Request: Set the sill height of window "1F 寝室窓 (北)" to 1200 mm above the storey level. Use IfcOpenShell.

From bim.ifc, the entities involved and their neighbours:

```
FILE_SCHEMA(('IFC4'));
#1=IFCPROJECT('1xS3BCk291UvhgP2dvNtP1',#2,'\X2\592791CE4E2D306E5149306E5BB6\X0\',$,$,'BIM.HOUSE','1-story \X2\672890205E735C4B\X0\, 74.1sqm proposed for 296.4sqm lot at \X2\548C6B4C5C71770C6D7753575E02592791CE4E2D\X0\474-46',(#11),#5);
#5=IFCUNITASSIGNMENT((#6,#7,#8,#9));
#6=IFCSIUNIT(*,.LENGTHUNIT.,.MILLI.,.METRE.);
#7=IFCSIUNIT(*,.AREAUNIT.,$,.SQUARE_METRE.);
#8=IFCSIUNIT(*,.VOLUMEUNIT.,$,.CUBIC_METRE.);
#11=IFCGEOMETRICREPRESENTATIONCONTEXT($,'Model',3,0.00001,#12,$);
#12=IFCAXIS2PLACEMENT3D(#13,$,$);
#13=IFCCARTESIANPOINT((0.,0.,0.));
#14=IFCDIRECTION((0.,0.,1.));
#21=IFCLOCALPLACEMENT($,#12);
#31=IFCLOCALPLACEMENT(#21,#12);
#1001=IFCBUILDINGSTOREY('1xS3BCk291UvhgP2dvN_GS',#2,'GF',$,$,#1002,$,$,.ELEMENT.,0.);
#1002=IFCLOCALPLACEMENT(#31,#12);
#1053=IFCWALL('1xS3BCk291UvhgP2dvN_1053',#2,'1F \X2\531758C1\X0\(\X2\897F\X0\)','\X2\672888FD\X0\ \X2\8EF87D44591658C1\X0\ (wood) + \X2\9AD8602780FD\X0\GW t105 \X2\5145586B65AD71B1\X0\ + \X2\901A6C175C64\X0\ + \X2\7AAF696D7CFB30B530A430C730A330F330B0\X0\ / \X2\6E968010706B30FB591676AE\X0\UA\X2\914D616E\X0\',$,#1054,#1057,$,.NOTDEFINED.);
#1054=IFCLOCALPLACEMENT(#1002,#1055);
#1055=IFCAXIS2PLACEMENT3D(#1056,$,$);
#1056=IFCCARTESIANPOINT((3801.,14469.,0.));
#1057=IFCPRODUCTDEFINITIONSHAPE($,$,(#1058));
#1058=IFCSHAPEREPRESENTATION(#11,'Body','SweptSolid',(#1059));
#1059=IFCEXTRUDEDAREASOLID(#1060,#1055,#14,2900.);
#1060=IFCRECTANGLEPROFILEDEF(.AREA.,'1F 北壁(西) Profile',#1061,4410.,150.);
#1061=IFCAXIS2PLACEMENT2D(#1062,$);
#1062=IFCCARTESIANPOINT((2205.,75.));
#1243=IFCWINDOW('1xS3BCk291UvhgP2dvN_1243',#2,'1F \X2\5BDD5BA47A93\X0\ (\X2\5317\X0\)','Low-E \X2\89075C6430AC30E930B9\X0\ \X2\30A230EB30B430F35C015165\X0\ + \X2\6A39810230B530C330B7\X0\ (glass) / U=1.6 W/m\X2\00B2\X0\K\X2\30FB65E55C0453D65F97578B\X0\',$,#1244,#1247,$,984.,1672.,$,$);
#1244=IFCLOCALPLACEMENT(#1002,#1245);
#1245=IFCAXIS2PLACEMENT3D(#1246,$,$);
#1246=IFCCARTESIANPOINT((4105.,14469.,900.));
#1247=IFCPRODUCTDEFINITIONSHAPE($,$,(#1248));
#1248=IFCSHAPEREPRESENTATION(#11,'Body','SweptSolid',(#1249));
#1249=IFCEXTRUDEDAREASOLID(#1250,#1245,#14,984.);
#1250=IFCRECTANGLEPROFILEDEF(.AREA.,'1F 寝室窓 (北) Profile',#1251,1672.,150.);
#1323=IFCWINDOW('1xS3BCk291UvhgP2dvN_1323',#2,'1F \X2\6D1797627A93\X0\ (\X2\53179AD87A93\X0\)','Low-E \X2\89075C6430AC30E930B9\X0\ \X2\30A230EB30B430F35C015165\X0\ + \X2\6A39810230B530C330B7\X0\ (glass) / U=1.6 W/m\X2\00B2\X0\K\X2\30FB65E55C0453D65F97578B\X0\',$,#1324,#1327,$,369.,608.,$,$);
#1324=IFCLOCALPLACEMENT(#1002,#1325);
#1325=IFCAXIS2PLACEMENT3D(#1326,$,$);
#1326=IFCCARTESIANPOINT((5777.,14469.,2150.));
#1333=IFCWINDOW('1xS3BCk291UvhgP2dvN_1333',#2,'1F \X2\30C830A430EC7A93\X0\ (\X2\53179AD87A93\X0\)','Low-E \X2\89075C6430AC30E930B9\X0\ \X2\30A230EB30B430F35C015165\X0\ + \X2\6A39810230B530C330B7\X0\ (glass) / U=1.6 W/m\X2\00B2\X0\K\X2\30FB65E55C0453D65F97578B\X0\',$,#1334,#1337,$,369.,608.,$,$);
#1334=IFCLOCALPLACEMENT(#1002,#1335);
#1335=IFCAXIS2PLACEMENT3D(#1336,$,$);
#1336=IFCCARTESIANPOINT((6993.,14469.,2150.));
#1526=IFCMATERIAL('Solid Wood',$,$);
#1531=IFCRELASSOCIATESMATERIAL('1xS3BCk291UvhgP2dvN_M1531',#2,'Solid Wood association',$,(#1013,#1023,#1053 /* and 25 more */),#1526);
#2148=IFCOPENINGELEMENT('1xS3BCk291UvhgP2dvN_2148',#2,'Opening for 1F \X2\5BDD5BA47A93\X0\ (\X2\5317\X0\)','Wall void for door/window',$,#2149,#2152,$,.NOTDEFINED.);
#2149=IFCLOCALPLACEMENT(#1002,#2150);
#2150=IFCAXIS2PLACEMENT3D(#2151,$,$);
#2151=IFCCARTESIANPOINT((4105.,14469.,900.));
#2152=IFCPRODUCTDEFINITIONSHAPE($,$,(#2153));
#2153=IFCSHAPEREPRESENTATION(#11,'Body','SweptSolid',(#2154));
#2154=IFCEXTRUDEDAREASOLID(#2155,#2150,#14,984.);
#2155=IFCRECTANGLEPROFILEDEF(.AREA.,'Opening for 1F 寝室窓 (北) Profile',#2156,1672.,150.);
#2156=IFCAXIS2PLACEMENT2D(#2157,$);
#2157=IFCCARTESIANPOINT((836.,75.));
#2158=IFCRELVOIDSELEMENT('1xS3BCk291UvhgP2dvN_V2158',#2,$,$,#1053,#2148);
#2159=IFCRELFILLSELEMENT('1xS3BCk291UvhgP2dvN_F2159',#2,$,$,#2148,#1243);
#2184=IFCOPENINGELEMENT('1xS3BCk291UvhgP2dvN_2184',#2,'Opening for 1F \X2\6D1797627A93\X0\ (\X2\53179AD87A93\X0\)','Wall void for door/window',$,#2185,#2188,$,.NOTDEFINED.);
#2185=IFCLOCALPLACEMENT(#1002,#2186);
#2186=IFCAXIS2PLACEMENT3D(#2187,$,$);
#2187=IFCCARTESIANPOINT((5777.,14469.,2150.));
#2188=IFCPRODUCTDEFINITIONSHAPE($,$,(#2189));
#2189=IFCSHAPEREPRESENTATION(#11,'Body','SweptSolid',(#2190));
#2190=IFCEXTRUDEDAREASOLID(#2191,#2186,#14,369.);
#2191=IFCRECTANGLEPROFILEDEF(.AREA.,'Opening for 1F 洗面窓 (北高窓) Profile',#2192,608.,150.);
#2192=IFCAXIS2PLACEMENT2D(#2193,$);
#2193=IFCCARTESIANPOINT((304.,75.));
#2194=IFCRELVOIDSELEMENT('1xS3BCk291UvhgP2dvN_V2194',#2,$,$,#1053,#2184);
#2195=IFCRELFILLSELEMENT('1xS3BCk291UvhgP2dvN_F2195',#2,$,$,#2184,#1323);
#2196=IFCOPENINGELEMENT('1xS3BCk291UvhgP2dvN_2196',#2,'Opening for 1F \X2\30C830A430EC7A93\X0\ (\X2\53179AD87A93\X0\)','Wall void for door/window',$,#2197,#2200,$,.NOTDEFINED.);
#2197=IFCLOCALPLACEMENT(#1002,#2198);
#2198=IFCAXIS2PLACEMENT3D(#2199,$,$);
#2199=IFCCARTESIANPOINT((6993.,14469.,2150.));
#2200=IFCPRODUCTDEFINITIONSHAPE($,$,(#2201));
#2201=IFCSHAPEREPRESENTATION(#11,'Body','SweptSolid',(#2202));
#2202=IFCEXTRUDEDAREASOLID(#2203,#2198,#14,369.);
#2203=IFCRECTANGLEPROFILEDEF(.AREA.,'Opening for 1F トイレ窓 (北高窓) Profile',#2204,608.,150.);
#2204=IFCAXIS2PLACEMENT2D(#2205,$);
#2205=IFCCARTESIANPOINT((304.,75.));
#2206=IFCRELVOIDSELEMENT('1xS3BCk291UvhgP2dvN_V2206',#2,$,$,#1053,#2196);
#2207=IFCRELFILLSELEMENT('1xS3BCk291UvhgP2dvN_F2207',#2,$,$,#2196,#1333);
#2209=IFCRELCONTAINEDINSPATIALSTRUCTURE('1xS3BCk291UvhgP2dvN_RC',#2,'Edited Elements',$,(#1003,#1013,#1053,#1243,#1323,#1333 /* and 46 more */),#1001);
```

```python
import numpy as np
import ifcopenshell
import ifcopenshell.api.geometry
import ifcopenshell.geom
import ifcopenshell.util.element
import ifcopenshell.util.placement
import ifcopenshell.util.shape
import ifcopenshell.util.unit

model = ifcopenshell.open("bim.ifc")
unit_scale = ifcopenshell.util.unit.calculate_unit_scale(model)

window = model.by_guid("1xS3BCk291UvhgP2dvN_1243")
opening = window.FillsVoids[0].RelatingOpeningElement
storey = ifcopenshell.util.element.get_container(window, ifc_class="IfcBuildingStorey")
level = ifcopenshell.util.placement.get_local_placement(storey.ObjectPlacement)[2, 3]

# The opening's origin need not be at the sill, so measure its lowest point.
shape = ifcopenshell.geom.create_shape(ifcopenshell.geom.settings(), opening)
bottom = ifcopenshell.util.shape.get_shape_bottom_elevation(shape, shape.geometry) / unit_scale
dz = level + 1200.0 - bottom

shift = np.array([0.0, 0.0, dz])
# The window is not placed relative to its opening, so move both.
for product in (opening, window):
    matrix = ifcopenshell.util.placement.get_local_placement(product.ObjectPlacement)
    matrix[:3, 3] += shift
    ifcopenshell.api.geometry.edit_object_placement(model, product=product, matrix=matrix, is_si=False)

print(f"moved by {dz * unit_scale:+.3f} m")

model.write("bim_rev.ifc")
```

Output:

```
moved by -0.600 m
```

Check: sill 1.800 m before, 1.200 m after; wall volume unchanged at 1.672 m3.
